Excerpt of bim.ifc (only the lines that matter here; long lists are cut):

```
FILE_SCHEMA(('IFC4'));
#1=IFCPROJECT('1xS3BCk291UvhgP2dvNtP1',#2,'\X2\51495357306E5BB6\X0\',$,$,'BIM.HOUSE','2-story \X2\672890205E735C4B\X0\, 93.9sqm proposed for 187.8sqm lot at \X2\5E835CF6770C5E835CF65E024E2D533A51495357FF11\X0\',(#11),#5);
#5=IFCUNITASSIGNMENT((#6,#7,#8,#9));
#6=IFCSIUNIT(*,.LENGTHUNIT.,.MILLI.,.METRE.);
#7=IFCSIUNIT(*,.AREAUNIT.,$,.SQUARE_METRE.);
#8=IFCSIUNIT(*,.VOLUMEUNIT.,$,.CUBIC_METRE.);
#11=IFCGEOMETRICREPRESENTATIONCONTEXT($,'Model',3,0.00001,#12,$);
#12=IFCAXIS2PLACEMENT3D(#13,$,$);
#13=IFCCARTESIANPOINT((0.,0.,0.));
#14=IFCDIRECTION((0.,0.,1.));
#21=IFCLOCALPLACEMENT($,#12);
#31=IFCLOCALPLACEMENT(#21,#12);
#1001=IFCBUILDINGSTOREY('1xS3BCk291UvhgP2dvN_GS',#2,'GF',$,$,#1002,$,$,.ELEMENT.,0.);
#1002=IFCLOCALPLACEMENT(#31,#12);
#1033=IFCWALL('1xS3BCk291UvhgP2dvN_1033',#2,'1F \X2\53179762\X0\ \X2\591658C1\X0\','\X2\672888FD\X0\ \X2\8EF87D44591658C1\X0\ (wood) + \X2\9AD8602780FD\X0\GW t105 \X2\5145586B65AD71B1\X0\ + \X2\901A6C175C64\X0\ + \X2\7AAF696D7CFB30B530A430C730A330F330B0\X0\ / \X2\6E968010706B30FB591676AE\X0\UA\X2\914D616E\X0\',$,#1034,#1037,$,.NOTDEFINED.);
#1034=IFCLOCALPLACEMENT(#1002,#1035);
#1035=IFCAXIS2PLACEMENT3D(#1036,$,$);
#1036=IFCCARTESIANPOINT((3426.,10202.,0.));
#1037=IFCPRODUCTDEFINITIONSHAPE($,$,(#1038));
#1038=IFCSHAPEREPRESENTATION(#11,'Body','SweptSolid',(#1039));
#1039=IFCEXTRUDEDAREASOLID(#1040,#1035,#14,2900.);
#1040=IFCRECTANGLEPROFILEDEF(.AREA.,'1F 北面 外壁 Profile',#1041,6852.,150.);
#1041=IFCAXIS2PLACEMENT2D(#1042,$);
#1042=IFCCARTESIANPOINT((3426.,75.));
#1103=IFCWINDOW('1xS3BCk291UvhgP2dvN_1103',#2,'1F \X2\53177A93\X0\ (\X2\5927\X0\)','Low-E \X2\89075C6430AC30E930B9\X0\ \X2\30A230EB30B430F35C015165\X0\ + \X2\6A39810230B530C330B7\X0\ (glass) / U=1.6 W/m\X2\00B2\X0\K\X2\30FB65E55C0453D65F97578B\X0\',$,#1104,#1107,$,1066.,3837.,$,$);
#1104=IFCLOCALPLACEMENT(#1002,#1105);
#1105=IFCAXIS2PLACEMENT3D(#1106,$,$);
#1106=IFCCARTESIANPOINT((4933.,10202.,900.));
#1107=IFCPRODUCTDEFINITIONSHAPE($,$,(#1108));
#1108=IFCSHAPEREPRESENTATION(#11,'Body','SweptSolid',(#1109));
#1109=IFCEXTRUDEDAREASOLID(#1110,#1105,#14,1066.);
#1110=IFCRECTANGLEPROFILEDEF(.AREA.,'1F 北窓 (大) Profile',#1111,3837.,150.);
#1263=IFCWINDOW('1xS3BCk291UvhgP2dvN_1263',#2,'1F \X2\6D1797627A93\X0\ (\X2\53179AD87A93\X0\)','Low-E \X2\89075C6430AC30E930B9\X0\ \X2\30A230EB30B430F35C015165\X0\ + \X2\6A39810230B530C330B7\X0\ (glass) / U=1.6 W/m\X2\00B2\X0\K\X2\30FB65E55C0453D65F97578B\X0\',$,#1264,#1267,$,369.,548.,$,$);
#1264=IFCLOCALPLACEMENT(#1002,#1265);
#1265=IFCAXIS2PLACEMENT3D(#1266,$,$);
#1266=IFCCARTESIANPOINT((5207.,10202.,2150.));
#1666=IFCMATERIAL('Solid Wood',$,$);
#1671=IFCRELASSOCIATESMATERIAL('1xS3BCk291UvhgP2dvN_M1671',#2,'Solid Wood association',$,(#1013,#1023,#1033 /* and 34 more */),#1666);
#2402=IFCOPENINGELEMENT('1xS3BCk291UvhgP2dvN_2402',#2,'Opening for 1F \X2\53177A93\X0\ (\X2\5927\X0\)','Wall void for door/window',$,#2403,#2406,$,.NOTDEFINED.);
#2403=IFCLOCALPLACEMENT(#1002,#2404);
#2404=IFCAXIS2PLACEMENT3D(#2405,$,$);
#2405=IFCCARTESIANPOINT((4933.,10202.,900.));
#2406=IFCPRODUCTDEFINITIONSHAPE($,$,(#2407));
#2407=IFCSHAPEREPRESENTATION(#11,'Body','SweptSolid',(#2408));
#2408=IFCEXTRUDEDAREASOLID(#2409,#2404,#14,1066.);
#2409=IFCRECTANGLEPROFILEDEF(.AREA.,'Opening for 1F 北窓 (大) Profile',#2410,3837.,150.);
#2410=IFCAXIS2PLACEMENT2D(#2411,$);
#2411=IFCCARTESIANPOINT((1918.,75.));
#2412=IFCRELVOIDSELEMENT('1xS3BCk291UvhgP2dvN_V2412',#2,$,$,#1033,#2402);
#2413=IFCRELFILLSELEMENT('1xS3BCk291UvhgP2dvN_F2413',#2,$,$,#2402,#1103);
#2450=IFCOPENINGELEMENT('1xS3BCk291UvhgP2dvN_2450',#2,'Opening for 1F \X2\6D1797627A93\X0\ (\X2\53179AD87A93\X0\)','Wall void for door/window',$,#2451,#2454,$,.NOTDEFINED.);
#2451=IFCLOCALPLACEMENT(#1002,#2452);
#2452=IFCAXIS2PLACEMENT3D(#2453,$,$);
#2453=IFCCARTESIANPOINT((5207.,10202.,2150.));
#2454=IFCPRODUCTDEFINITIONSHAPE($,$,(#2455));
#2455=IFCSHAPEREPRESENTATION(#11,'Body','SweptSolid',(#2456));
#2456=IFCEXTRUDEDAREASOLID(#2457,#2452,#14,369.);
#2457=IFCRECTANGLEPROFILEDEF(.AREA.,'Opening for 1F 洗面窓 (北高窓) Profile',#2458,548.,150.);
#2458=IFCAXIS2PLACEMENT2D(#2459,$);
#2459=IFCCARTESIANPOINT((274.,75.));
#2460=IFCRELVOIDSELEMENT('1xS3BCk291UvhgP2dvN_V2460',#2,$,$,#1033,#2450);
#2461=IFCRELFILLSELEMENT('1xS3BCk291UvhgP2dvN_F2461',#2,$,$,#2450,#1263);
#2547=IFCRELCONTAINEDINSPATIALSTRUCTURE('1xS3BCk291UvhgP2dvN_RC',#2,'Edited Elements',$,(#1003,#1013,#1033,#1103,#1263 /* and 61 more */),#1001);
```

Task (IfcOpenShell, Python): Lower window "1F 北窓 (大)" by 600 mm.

```python
import numpy as np
import ifcopenshell
import ifcopenshell.api.geometry
import ifcopenshell.util.placement
import ifcopenshell.util.unit

model = ifcopenshell.open("bim.ifc")
unit_scale = ifcopenshell.util.unit.calculate_unit_scale(model)

window = model.by_guid("1xS3BCk291UvhgP2dvN_1103")
opening = window.FillsVoids[0].RelatingOpeningElement
dz = -0.6 / unit_scale

shift = np.array([0.0, 0.0, dz])
# The window is not placed relative to its opening, so move both.
for product in (opening, window):
    matrix = ifcopenshell.util.placement.get_local_placement(product.ObjectPlacement)
    matrix[:3, 3] += shift
    ifcopenshell.api.geometry.edit_object_placement(model, product=product, matrix=matrix, is_si=False)

print(f"moved by {dz * unit_scale:+.3f} m")

model.write("bim-out.ifc")
```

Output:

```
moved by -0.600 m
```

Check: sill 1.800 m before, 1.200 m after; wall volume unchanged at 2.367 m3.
